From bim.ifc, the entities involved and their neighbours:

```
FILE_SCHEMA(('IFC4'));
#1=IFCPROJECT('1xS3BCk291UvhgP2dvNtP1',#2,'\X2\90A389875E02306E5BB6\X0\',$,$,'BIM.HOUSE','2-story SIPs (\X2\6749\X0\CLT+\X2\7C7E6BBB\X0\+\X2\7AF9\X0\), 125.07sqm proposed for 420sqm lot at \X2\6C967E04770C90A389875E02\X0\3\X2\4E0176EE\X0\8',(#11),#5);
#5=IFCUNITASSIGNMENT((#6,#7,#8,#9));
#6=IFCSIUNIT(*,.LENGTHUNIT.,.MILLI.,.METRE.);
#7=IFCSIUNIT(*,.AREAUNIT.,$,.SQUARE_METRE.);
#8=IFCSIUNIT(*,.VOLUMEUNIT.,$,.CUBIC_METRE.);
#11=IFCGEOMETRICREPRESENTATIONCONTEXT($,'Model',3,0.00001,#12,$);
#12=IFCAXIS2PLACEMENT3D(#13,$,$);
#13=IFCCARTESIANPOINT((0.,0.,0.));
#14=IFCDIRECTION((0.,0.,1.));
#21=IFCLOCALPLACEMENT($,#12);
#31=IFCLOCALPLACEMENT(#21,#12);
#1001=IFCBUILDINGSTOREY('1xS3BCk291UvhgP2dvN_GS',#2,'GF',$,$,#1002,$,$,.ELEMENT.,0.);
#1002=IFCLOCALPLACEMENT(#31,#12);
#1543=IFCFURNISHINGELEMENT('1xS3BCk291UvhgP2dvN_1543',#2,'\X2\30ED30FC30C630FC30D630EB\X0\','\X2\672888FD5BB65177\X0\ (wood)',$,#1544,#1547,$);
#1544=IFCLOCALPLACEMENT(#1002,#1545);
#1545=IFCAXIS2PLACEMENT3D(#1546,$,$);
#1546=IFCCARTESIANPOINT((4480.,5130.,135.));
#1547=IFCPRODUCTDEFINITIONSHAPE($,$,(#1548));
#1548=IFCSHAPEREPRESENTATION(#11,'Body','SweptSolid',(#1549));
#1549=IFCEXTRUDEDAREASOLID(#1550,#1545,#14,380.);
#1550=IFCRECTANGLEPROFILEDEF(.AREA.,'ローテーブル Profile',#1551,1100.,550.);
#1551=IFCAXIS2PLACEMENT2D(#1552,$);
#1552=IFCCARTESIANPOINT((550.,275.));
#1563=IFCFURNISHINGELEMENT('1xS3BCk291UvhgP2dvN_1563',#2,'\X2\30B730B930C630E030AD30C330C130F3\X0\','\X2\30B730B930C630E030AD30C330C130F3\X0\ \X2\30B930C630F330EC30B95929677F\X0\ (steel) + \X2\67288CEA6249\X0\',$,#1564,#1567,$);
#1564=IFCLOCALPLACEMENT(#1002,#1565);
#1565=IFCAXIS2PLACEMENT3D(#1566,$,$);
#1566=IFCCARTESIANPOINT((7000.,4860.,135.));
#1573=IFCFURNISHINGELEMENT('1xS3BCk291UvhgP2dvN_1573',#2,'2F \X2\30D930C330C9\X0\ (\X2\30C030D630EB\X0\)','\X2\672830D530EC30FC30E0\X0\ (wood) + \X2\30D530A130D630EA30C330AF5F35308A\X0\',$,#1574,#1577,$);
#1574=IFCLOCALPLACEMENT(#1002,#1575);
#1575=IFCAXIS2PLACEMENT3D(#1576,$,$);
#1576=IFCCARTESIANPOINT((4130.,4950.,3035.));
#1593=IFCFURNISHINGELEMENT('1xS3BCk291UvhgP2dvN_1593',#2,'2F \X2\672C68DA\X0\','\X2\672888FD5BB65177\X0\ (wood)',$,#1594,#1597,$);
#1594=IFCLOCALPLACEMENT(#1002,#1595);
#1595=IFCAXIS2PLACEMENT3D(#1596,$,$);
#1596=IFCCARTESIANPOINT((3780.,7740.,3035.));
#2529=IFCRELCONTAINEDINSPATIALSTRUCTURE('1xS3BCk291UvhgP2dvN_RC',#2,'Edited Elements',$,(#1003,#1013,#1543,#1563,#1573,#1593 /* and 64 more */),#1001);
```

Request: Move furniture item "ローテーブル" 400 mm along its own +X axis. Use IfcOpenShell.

```python
import ifcopenshell
import ifcopenshell.api.geometry
import ifcopenshell.util.placement

model = ifcopenshell.open("bim.ifc")

item = model.by_guid("1xS3BCk291UvhgP2dvN_1543")
matrix = ifcopenshell.util.placement.get_local_placement(item.ObjectPlacement)
matrix[:3, 3] += matrix[:3, 0] * 400.0
ifcopenshell.api.geometry.edit_object_placement(model, product=item, matrix=matrix, is_si=False)

print(ifcopenshell.util.placement.get_local_placement(item.ObjectPlacement).round(3) + 0.0)

model.write("bim-out.ifc")
```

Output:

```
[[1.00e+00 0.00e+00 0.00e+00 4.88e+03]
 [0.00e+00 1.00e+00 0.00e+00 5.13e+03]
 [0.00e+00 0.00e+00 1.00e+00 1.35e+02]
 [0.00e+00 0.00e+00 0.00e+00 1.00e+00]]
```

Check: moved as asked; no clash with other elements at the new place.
